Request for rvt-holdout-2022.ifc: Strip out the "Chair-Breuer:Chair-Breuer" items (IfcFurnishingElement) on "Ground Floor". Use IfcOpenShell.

First a look at what the model holds.

```python
import ifcopenshell
import ifcopenshell.util.element

model = ifcopenshell.open("rvt-holdout-2022.ifc")
print(model.schema)
storey = next(s for s in model.by_type("IfcBuildingStorey") if s.Name == "Ground Floor")
furniture = [e for e in ifcopenshell.util.element.get_decomposition(storey) if e.is_a("IfcFurnishingElement")]
seen = {}
for e in furniture:
    element_type = ifcopenshell.util.element.get_type(e)
    name = element_type.Name if element_type not in (None, e) else None
    seen[name] = seen.get(name, 0) + 1
for name, count in sorted(seen.items(), key=str):
    print(count, "x", name)
```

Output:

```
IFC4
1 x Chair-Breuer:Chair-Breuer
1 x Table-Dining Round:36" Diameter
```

```python
import ifcopenshell
import ifcopenshell.api.root
import ifcopenshell.util.element

model = ifcopenshell.open("rvt-holdout-2022.ifc")

storey = next(s for s in model.by_type("IfcBuildingStorey") if s.Name == "Ground Floor")
furniture = [e for e in ifcopenshell.util.element.get_decomposition(storey) if e.is_a("IfcFurnishingElement")]
targets = [e for e in furniture if (t := ifcopenshell.util.element.get_type(e)) not in (None, e) and t.Name == "Chair-Breuer:Chair-Breuer"]

for e in targets:
    ifcopenshell.api.root.remove_product(model, product=e)
print(len(targets), "removed")

model.write("rvt-holdout-2022_v2.ifc")
```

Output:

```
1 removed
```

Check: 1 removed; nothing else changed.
